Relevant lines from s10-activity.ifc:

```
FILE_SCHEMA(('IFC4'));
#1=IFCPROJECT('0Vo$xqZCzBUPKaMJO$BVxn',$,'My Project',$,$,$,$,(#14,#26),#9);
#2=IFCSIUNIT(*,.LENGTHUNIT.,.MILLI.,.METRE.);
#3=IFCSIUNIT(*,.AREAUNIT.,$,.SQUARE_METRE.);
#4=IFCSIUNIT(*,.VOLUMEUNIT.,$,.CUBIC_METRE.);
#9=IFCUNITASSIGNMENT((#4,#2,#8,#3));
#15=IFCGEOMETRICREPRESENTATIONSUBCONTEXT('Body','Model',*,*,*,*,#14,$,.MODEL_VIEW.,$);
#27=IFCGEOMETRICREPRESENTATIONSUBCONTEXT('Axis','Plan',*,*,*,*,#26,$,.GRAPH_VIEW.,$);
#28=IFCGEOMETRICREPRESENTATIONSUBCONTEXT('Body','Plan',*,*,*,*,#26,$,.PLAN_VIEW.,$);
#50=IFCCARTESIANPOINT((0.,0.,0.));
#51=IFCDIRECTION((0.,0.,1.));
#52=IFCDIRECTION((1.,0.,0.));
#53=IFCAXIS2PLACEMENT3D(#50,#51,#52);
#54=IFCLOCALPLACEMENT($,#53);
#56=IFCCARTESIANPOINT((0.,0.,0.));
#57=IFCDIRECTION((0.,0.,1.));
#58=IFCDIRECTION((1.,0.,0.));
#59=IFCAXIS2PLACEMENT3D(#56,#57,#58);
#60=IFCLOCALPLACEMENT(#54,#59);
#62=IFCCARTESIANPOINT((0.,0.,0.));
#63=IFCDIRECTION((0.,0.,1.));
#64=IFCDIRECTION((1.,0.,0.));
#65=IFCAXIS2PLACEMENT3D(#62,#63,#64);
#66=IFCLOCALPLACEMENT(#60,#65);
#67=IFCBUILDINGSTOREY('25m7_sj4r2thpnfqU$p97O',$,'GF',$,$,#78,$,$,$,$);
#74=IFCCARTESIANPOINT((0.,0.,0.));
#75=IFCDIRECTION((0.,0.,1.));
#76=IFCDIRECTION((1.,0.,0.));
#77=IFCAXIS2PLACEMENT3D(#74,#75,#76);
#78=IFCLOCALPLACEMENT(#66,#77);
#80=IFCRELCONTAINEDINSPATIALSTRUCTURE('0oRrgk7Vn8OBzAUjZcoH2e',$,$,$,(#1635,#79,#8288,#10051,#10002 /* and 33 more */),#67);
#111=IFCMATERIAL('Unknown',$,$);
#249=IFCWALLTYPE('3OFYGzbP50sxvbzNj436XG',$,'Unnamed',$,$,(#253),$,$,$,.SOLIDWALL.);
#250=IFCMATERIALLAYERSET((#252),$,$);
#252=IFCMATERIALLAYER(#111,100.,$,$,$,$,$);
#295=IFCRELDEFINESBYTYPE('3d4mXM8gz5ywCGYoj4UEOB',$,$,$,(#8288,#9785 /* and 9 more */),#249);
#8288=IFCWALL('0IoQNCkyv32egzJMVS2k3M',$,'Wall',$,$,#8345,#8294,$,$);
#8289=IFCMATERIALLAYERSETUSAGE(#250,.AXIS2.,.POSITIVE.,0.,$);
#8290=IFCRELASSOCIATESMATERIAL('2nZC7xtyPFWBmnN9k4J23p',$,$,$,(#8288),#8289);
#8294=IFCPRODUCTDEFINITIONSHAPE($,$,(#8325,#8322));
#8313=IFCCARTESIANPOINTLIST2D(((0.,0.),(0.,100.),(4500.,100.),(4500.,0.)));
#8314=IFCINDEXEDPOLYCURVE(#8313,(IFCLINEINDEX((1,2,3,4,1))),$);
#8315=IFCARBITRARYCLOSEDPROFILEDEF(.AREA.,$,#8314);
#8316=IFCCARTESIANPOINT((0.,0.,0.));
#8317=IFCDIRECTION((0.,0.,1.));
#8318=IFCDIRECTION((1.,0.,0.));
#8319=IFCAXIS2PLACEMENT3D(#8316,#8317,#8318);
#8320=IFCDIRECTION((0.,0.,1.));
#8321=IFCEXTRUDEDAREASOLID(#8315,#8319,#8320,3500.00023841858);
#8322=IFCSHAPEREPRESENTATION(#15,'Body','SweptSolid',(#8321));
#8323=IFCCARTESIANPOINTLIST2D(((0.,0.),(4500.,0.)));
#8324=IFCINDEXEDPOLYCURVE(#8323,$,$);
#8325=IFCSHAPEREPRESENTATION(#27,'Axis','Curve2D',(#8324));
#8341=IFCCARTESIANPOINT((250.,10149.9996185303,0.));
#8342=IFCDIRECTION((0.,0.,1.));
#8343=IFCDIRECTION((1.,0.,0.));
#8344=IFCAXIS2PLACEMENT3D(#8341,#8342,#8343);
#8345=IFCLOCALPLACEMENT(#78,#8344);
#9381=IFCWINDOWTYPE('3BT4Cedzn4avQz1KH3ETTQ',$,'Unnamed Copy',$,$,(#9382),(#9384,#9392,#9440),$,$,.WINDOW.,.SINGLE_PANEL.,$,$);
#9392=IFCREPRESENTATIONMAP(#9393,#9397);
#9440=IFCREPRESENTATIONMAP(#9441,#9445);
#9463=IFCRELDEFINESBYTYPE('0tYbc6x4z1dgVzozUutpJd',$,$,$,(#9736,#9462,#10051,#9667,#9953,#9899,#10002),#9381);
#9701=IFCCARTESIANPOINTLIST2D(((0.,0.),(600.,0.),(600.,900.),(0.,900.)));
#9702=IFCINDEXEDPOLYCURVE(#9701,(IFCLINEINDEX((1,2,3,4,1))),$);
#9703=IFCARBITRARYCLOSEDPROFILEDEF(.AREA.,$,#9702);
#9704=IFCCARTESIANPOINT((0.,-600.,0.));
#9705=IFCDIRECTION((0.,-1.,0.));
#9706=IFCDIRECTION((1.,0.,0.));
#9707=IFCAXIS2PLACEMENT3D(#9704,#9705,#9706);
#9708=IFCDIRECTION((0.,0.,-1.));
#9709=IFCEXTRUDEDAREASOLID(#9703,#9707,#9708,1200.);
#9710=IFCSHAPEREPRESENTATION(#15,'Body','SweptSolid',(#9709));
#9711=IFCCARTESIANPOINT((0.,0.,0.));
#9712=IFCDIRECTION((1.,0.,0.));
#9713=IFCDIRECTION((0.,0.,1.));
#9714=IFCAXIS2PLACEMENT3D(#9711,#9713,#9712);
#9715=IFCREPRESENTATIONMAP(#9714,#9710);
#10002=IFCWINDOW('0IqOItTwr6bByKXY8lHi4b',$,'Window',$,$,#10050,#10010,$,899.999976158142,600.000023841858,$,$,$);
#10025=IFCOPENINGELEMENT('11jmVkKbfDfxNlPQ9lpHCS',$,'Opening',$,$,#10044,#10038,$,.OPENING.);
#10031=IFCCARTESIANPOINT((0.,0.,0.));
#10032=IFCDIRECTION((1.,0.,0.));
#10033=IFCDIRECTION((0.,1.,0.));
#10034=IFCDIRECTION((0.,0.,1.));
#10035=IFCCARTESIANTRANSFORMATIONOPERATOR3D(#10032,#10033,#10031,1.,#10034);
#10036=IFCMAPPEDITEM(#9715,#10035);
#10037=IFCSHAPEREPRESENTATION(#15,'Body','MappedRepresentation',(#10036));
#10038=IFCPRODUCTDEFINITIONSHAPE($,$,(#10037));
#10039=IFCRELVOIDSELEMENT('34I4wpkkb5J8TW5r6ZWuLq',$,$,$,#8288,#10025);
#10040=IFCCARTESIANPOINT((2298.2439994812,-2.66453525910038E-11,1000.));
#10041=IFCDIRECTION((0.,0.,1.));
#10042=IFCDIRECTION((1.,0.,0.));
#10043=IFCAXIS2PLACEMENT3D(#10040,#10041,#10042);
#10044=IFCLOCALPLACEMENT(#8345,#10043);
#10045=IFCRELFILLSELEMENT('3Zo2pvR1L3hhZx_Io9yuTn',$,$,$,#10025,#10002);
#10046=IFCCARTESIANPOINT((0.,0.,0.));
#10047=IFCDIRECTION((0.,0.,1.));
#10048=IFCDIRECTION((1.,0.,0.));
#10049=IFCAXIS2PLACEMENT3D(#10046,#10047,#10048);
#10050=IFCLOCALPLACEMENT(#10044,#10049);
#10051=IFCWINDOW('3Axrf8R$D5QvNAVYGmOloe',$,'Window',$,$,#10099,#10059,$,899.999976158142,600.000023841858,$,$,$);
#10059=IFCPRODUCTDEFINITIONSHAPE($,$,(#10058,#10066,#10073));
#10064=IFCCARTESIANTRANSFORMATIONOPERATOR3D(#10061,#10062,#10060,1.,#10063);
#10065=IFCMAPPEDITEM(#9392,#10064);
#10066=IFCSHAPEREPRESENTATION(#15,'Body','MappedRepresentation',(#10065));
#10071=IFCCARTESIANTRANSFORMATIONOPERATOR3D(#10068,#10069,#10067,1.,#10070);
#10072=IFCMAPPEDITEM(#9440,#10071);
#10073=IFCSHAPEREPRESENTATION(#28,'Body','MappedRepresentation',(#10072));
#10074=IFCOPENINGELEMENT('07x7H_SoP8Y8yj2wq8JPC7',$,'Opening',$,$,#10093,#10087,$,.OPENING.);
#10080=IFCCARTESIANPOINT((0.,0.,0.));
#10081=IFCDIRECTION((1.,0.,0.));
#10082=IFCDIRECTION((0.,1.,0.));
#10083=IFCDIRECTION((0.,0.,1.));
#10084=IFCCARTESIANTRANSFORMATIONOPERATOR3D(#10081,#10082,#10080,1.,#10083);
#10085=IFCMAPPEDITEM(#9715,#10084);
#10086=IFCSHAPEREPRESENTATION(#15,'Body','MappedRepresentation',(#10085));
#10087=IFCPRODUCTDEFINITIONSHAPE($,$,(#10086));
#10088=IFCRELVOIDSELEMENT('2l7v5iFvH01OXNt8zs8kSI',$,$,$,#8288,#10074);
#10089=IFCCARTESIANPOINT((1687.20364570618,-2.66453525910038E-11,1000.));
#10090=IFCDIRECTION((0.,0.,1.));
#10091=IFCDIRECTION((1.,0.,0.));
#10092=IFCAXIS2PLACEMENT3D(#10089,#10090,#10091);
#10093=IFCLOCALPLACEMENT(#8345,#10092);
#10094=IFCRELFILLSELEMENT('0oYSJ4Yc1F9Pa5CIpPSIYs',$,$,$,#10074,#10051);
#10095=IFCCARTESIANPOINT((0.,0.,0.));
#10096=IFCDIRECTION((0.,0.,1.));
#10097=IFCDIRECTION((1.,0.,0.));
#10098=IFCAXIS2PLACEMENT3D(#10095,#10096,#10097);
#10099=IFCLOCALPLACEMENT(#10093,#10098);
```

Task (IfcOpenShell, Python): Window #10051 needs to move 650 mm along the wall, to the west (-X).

```python
import ifcopenshell
import ifcopenshell.api.geometry
import ifcopenshell.util.placement

model = ifcopenshell.open("s10-activity.ifc")

window = model.by_id(10051)
opening = window.FillsVoids[0].RelatingOpeningElement
wall = opening.VoidsElements[0].RelatingBuildingElement

wall_matrix = ifcopenshell.util.placement.get_local_placement(wall.ObjectPlacement)
shift = wall_matrix[:3, 0] * -650.0
before = ifcopenshell.util.placement.get_local_placement(window.ObjectPlacement)[:3, 3].copy()

# The window is placed relative to its opening, so it follows when the opening moves.
matrix = ifcopenshell.util.placement.get_local_placement(opening.ObjectPlacement)
matrix[:3, 3] += shift
ifcopenshell.api.geometry.edit_object_placement(
    model, product=opening, matrix=matrix, is_si=False, should_transform_children=True
)

after = ifcopenshell.util.placement.get_local_placement(window.ObjectPlacement)[:3, 3]
print("window moved by", (after - before).round(3) + 0.0)

model.write("s10-activity_v2.ifc")
```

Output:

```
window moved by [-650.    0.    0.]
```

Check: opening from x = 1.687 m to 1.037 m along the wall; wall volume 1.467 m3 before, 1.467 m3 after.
